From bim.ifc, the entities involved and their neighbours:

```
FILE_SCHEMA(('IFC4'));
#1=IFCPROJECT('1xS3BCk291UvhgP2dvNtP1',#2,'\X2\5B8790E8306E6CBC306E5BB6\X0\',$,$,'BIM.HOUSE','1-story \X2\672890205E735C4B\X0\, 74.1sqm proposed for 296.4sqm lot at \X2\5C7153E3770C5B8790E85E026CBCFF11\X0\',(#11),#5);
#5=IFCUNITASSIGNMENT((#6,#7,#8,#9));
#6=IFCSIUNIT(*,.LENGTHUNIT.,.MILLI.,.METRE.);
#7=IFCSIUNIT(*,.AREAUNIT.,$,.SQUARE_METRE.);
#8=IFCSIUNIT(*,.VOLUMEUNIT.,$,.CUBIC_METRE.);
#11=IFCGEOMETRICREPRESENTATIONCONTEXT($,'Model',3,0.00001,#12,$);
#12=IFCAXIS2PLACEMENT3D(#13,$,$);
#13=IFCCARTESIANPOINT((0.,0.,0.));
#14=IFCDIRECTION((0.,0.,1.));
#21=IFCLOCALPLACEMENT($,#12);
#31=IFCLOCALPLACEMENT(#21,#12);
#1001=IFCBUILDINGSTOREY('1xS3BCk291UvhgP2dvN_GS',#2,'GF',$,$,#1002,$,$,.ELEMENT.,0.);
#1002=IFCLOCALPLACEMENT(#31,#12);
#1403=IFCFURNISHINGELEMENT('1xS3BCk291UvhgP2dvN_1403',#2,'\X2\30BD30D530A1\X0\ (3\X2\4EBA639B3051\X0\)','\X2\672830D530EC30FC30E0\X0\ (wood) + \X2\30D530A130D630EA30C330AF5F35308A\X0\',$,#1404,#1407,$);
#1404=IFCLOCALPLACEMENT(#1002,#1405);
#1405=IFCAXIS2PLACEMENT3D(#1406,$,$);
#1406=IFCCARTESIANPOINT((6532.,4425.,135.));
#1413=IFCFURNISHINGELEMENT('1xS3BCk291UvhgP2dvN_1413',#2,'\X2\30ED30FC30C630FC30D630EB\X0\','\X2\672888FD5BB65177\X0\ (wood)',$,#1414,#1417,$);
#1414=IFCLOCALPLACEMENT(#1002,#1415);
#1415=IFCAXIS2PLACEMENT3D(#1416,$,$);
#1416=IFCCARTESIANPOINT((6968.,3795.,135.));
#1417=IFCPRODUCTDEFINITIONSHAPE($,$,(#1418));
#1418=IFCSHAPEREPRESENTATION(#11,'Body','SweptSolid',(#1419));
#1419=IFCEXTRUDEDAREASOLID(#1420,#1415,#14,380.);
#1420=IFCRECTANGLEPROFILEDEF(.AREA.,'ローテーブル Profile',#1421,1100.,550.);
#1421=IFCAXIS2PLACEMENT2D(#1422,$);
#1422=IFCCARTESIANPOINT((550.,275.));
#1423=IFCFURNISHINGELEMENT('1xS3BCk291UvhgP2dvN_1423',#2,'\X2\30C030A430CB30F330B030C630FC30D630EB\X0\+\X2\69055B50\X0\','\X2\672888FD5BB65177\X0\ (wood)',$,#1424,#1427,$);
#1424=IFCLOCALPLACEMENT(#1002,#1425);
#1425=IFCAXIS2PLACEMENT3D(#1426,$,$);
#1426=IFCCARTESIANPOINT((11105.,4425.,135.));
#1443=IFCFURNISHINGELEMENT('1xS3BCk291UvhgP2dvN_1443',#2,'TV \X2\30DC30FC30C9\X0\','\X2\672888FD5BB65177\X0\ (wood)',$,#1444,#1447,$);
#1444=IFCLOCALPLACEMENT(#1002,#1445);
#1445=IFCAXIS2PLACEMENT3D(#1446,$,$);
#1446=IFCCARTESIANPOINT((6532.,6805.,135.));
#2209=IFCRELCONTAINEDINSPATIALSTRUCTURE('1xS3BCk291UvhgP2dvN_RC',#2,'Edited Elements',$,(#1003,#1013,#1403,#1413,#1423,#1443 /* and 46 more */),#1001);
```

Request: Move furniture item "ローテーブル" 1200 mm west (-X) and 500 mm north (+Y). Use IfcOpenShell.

```python
import ifcopenshell
import ifcopenshell.api.geometry
import ifcopenshell.util.placement

model = ifcopenshell.open("bim.ifc")

item = model.by_guid("1xS3BCk291UvhgP2dvN_1413")
matrix = ifcopenshell.util.placement.get_local_placement(item.ObjectPlacement)
matrix[0, 3] -= 1200.0
matrix[1, 3] += 500.0
ifcopenshell.api.geometry.edit_object_placement(model, product=item, matrix=matrix, is_si=False)

print(ifcopenshell.util.placement.get_local_placement(item.ObjectPlacement).round(3) + 0.0)

model.write("bim-out.ifc")
```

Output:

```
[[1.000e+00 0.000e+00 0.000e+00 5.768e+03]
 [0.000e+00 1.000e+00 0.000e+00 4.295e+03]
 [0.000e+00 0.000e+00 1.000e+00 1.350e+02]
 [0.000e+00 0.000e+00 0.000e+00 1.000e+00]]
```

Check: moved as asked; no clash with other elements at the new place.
